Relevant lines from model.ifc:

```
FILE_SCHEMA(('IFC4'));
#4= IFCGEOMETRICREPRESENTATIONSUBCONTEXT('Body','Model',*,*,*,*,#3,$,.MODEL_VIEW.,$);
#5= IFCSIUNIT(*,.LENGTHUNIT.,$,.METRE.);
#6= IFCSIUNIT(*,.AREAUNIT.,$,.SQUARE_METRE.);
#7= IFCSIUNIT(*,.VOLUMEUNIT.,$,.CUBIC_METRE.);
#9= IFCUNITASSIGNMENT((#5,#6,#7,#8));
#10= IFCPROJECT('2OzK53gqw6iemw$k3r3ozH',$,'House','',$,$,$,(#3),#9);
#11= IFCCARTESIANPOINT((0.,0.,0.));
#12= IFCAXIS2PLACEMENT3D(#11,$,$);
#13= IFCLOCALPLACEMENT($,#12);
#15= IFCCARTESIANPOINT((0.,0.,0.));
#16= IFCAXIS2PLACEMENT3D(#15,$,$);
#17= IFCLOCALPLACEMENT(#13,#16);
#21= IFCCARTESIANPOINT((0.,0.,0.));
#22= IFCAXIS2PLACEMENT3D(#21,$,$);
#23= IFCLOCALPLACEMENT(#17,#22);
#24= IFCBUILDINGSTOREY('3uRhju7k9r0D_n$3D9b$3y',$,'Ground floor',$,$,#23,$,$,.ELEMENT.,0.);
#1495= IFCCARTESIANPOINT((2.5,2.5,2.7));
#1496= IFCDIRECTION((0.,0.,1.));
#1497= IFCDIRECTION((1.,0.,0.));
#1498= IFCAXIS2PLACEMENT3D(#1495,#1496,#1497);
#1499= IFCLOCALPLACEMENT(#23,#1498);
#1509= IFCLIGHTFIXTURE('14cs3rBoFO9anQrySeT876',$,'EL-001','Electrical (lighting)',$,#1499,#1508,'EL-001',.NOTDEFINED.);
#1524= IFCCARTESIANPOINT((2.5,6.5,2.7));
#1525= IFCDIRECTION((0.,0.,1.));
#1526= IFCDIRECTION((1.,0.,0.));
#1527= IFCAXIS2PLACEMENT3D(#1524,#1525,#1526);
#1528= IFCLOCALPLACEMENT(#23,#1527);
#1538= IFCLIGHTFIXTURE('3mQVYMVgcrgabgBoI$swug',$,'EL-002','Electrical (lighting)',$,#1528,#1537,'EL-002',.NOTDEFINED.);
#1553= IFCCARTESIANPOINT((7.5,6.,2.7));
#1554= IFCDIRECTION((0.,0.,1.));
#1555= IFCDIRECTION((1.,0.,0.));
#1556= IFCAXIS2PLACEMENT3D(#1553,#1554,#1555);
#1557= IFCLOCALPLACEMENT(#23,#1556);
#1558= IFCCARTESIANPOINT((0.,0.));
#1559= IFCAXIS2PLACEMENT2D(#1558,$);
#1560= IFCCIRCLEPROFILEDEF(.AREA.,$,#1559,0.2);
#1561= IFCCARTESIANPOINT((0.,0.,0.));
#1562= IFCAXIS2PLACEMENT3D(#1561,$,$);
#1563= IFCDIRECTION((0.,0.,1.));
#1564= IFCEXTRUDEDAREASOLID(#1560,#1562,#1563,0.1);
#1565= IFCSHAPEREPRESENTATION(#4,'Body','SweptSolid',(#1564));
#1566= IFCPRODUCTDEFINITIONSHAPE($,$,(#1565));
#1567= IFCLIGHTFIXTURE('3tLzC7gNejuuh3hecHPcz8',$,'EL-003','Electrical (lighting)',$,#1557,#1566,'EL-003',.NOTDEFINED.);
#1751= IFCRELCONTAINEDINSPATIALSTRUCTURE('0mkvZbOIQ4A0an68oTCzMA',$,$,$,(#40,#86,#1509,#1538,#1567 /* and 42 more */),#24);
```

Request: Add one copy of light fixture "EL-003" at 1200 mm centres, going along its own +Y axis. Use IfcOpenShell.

```python
import ifcopenshell
import ifcopenshell.api.geometry
import ifcopenshell.api.root
import ifcopenshell.util.element
import ifcopenshell.util.placement
import ifcopenshell.util.unit

model = ifcopenshell.open("model.ifc")
unit_scale = ifcopenshell.util.unit.calculate_unit_scale(model)

source = model.by_guid("3tLzC7gNejuuh3hecHPcz8")
base = ifcopenshell.util.placement.get_local_placement(source.ObjectPlacement)
step = base[:3, 1] * 1.2 / unit_scale

for i in range(1, 2):
    copy = ifcopenshell.api.root.copy_class(model, product=source)
    copy.Representation = ifcopenshell.util.element.copy_deep(
        model, source.Representation, exclude=["IfcGeometricRepresentationContext", "IfcRepresentationMap"]
    )
    copy.Tag = None
    matrix = base.copy()
    matrix[:3, 3] += i * step
    print("added at", matrix[:3, 3].round(3) + 0.0)
    ifcopenshell.api.geometry.edit_object_placement(model, product=copy, matrix=matrix, is_si=False)

model.write("model_updated.ifc")
```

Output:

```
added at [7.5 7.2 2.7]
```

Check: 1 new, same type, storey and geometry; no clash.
